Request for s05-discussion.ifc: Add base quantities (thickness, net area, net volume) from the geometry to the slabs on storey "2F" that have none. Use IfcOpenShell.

First a look at what the model holds.

```python
import ifcopenshell
import ifcopenshell.util.element
import ifcopenshell.util.unit

model = ifcopenshell.open("s05-discussion.ifc")
print(model.schema)
for unit_type in ("LENGTHUNIT", "AREAUNIT", "VOLUMEUNIT"):
    print(unit_type, ifcopenshell.util.unit.calculate_unit_scale(model, unit_type))
storey = next(s for s in model.by_type("IfcBuildingStorey") if s.Name == "2F")
slabs = [e for e in ifcopenshell.util.element.get_decomposition(storey) if e.is_a("IfcSlab")]
for e in sorted(slabs, key=lambda e: e.id()):
    print(e.id(), e.is_a(), e.Name, list(ifcopenshell.util.element.get_psets(e, qtos_only=True)), sep=" | ")
```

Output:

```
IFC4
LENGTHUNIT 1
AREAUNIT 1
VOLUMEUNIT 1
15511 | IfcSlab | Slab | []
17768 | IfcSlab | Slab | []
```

```python
import ifcopenshell
import ifcopenshell.api.pset
import ifcopenshell.geom
import ifcopenshell.util.element
import ifcopenshell.util.shape
import ifcopenshell.util.unit

model = ifcopenshell.open("s05-discussion.ifc")
unit_scale = ifcopenshell.util.unit.calculate_unit_scale(model)
area_scale = ifcopenshell.util.unit.calculate_unit_scale(model, "AREAUNIT")
volume_scale = ifcopenshell.util.unit.calculate_unit_scale(model, "VOLUMEUNIT")
settings = ifcopenshell.geom.settings()

storey = next(s for s in model.by_type("IfcBuildingStorey") if s.Name == "2F")
slabs = [e for e in ifcopenshell.util.element.get_decomposition(storey) if e.is_a("IfcSlab")]

for e in sorted(slabs, key=lambda e: e.id()):
    if ifcopenshell.util.element.get_psets(e, qtos_only=True, should_inherit=False):
        continue
    # Geometry comes back in metres, in the element's own axes.
    shape = ifcopenshell.geom.create_shape(settings, e)
    values = {
        "Width": ifcopenshell.util.shape.get_z(shape.geometry) / unit_scale,
        "NetArea": ifcopenshell.util.shape.get_footprint_area(shape.geometry) / area_scale,
        "NetVolume": ifcopenshell.util.shape.get_volume(shape.geometry) / volume_scale,
    }
    qto = ifcopenshell.api.pset.add_qto(model, product=e, name="Qto_SlabBaseQuantities")
    ifcopenshell.api.pset.edit_qto(model, qto=qto, properties=values)
    print(e.id(), {k: round(v, 3) for k, v in values.items()})

model.write("s05-discussion_edited.ifc")
```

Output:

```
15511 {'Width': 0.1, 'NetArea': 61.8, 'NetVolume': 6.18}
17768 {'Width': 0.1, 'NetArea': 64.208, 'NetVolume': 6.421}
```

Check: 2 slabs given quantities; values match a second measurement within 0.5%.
